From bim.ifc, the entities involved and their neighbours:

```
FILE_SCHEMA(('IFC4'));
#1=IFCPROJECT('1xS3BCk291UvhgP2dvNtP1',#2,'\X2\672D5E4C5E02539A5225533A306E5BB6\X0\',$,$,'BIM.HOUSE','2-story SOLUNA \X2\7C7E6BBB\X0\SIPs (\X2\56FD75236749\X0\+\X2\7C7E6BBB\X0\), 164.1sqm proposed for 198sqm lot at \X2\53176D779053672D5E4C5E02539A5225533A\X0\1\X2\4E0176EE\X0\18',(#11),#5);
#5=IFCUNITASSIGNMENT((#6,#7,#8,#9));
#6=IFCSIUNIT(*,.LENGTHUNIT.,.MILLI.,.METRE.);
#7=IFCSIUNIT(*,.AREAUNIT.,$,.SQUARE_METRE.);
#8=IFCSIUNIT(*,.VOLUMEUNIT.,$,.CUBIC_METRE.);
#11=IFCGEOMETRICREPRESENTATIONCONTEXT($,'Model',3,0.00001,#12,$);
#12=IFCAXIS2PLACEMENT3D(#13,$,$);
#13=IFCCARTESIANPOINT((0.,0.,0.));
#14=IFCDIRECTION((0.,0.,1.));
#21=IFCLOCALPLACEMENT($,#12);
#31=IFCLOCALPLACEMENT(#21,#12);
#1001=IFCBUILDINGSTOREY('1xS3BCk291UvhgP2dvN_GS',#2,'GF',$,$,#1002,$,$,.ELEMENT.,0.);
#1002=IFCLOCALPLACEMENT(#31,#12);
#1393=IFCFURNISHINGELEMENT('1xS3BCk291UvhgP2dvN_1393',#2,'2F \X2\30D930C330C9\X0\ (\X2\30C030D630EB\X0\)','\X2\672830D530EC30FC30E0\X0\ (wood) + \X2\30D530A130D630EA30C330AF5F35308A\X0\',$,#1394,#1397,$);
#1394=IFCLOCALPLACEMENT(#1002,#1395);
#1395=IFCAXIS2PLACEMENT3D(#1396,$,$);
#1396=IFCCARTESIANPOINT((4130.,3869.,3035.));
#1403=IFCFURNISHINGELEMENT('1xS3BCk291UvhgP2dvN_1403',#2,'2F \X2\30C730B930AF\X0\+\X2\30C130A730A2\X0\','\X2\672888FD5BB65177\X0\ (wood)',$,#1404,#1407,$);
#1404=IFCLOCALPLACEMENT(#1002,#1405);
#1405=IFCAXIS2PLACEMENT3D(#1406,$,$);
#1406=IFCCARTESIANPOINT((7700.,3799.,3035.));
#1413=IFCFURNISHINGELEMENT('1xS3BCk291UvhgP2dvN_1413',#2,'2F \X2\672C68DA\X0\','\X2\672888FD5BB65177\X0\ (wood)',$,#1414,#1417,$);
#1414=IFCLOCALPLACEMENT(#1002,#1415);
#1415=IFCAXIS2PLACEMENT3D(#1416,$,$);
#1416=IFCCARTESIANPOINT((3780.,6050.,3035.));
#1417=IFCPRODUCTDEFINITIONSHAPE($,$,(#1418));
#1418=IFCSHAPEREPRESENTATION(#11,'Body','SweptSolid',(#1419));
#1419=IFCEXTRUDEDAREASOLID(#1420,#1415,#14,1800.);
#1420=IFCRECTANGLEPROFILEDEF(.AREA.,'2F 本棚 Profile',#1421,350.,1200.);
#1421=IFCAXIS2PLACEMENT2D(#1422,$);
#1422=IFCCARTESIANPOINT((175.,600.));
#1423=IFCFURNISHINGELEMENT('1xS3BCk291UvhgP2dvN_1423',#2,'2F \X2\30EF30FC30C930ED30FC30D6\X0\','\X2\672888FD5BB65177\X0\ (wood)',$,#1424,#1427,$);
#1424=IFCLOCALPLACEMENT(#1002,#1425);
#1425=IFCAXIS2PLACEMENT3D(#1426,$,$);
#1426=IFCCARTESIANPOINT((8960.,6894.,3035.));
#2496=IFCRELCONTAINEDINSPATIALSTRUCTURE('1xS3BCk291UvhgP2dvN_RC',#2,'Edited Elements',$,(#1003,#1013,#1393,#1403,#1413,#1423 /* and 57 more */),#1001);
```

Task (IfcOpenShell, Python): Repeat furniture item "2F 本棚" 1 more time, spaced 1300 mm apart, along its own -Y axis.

```python
import ifcopenshell
import ifcopenshell.api.geometry
import ifcopenshell.api.root
import ifcopenshell.util.element
import ifcopenshell.util.placement

model = ifcopenshell.open("bim.ifc")


def reuse_history(source, copy):
    """copy_class also copies each property set's owner history, people and application; keep the originals."""
    for rel in copy.IsDefinedBy:
        if rel.is_a("IfcRelDefinesByProperties") and (history := rel.RelatingPropertyDefinition.OwnerHistory):
            rel.RelatingPropertyDefinition.OwnerHistory = source.OwnerHistory
            ifcopenshell.util.element.remove_deep2(model, history)


source = model.by_guid("1xS3BCk291UvhgP2dvN_1413")
base = ifcopenshell.util.placement.get_local_placement(source.ObjectPlacement)
step = -base[:3, 1] * 1300.0

for i in range(1, 2):
    copy = ifcopenshell.api.root.copy_class(model, product=source)
    copy.Representation = ifcopenshell.util.element.copy_deep(
        model, source.Representation, exclude=["IfcGeometricRepresentationContext", "IfcRepresentationMap"]
    )
    reuse_history(source, copy)
    matrix = base.copy()
    matrix[:3, 3] += i * step
    print("added at", matrix[:3, 3].round(3) + 0.0)
    ifcopenshell.api.geometry.edit_object_placement(model, product=copy, matrix=matrix, is_si=False)

model.write("bim_rev.ifc")
```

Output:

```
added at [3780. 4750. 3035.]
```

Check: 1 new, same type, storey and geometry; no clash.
